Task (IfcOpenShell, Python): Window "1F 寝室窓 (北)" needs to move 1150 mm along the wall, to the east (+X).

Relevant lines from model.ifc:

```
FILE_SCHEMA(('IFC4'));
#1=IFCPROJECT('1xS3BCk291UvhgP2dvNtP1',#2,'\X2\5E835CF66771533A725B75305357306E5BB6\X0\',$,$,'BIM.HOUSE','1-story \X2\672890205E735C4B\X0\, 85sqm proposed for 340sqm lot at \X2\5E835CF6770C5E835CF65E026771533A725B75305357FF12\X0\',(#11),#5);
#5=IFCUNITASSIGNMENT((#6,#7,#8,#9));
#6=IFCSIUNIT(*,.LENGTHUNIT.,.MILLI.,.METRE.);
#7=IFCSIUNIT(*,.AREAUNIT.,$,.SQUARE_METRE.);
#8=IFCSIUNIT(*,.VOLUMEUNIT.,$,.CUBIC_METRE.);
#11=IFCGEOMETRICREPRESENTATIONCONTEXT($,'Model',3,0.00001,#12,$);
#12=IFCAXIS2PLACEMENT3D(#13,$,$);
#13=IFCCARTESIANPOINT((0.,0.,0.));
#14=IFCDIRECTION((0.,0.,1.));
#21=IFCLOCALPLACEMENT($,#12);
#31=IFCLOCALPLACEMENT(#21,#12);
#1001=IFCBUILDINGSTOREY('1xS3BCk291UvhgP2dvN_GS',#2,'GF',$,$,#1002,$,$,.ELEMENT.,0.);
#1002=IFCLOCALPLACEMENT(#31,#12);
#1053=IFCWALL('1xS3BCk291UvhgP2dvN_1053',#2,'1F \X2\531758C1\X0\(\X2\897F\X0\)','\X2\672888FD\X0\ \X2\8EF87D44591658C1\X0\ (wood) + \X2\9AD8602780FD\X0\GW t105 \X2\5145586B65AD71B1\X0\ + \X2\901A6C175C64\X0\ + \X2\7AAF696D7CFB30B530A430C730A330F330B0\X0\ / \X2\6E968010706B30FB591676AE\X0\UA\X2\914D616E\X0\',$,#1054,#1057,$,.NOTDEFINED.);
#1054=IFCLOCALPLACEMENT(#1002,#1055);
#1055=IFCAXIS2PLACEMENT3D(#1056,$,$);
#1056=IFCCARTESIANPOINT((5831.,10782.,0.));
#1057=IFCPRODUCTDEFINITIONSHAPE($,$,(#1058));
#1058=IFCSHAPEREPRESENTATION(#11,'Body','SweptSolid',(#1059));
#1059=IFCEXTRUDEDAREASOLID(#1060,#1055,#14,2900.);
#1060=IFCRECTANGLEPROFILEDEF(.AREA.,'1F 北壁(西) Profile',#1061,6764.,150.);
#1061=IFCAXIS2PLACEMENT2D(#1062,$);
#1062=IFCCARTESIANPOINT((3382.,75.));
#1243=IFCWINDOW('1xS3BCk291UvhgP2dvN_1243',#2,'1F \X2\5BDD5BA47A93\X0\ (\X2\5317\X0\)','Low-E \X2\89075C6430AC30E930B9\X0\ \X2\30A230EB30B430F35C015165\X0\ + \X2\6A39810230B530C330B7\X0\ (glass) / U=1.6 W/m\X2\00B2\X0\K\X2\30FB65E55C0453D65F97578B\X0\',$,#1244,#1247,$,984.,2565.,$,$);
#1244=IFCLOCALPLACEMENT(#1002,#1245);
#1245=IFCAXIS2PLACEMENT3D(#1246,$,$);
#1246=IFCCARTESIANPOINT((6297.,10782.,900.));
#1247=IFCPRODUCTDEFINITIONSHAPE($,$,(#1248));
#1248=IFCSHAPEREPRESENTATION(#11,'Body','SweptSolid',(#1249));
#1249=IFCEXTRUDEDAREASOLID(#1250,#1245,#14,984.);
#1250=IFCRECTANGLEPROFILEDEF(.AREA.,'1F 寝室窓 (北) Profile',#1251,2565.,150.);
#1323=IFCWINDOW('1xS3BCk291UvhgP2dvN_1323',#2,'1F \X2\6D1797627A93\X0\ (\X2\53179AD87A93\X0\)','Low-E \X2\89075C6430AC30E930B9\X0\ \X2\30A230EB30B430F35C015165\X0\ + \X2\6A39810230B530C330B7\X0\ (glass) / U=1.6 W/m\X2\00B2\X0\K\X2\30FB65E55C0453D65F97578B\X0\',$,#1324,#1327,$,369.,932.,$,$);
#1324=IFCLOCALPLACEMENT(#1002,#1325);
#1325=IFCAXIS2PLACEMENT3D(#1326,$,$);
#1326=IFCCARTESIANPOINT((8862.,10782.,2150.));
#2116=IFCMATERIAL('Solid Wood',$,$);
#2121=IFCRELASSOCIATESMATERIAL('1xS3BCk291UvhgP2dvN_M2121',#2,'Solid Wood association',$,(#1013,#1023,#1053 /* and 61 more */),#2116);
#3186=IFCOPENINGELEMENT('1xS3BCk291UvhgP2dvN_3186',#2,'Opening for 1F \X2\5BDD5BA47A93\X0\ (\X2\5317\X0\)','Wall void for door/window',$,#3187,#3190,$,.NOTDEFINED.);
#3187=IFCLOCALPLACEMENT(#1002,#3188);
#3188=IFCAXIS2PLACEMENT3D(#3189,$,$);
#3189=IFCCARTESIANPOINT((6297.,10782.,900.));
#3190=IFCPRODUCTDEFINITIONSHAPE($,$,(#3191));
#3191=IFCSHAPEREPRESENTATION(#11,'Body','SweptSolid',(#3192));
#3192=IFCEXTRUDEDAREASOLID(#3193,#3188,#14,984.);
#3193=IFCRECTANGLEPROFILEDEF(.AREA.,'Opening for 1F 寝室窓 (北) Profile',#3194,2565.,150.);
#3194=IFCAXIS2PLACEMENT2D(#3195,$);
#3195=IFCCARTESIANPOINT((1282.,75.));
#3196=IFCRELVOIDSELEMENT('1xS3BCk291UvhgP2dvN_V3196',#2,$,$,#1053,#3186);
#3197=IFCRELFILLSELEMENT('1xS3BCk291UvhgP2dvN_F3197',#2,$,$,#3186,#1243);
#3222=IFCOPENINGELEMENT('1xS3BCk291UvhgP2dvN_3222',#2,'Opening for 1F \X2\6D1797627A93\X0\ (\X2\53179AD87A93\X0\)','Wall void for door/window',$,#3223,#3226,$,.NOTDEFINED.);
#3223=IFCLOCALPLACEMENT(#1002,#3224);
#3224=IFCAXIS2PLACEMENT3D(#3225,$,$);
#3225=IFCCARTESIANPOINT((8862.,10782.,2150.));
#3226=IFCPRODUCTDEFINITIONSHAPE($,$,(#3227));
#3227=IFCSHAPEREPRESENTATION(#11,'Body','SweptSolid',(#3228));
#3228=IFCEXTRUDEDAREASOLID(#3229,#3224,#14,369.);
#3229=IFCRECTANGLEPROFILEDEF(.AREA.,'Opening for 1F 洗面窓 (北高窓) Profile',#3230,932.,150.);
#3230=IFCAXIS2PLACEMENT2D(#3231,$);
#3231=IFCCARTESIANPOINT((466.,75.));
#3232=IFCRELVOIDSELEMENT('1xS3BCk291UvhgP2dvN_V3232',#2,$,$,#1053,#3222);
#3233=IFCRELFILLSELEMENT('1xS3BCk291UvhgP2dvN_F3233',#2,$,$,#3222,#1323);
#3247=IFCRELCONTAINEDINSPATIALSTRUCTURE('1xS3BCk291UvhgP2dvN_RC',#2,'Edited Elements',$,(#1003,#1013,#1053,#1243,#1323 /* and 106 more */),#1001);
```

```python
import ifcopenshell
import ifcopenshell.api.geometry
import ifcopenshell.util.placement

model = ifcopenshell.open("model.ifc")

window = model.by_guid("1xS3BCk291UvhgP2dvN_1243")
opening = window.FillsVoids[0].RelatingOpeningElement
wall = opening.VoidsElements[0].RelatingBuildingElement

wall_matrix = ifcopenshell.util.placement.get_local_placement(wall.ObjectPlacement)
shift = wall_matrix[:3, 0] * 1150.0
before = ifcopenshell.util.placement.get_local_placement(window.ObjectPlacement)[:3, 3].copy()

# The window is not placed relative to its opening, so move both.
for product in (opening, window):
    matrix = ifcopenshell.util.placement.get_local_placement(product.ObjectPlacement)
    matrix[:3, 3] += shift
    ifcopenshell.api.geometry.edit_object_placement(model, product=product, matrix=matrix, is_si=False)

after = ifcopenshell.util.placement.get_local_placement(window.ObjectPlacement)[:3, 3]
print("window moved by", (after - before).round(3) + 0.0)

model.write("model_edited.ifc")
```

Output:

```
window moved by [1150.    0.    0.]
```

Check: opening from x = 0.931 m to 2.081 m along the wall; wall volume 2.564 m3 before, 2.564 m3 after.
